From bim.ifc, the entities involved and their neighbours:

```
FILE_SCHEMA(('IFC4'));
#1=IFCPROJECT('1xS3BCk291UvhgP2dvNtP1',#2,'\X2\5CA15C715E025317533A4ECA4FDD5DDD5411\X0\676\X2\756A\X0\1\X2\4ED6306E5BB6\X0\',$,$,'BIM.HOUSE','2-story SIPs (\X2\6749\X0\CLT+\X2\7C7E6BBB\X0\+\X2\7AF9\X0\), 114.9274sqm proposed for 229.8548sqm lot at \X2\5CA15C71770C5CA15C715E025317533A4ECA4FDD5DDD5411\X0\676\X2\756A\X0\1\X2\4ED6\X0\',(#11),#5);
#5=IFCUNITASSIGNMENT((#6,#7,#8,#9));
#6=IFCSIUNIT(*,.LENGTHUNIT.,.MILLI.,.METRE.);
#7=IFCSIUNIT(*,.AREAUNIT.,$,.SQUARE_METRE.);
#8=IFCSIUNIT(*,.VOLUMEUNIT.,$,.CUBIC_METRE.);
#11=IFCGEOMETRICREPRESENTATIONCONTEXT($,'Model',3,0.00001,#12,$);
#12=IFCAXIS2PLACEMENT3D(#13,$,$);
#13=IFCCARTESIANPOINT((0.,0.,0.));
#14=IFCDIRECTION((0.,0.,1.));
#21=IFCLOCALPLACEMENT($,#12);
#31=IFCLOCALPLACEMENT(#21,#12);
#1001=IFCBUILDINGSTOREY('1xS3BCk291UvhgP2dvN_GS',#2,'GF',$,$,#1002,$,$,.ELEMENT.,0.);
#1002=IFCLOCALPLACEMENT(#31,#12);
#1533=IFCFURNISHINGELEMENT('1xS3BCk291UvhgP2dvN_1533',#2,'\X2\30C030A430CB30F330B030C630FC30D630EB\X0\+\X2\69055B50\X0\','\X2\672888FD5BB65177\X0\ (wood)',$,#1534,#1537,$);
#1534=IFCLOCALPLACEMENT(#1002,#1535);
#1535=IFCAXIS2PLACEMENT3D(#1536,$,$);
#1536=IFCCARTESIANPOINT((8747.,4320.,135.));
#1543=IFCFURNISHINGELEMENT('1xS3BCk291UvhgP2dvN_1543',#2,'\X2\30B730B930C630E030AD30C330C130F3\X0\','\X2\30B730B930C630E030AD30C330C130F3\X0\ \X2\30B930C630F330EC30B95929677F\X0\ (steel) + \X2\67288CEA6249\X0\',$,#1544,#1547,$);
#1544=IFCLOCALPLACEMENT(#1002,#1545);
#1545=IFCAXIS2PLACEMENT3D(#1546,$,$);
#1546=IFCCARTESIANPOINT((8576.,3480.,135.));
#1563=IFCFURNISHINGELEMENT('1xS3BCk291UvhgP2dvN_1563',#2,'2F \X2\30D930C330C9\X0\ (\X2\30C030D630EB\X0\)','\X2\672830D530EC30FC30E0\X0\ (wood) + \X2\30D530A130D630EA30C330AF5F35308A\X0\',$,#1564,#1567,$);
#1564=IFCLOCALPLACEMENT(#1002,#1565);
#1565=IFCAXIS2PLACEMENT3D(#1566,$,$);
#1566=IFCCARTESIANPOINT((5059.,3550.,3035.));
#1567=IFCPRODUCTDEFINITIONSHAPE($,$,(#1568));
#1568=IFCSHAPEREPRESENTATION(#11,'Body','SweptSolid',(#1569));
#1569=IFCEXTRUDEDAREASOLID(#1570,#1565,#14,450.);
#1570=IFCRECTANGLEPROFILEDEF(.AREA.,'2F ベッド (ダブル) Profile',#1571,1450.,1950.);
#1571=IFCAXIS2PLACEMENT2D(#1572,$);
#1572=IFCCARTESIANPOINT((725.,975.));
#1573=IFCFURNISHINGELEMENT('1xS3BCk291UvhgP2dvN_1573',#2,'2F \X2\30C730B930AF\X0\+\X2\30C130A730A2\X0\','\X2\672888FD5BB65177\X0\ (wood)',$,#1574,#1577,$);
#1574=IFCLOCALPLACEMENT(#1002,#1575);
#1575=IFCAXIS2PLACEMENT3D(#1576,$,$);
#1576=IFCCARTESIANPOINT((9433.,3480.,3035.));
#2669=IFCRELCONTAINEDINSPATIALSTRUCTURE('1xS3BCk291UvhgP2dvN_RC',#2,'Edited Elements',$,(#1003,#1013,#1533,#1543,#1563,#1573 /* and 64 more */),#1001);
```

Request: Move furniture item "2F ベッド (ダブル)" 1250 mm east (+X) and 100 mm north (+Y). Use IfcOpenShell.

```python
import ifcopenshell
import ifcopenshell.api.geometry
import ifcopenshell.util.placement
import ifcopenshell.util.unit

model = ifcopenshell.open("bim.ifc")
unit_scale = ifcopenshell.util.unit.calculate_unit_scale(model)

item = model.by_guid("1xS3BCk291UvhgP2dvN_1563")
matrix = ifcopenshell.util.placement.get_local_placement(item.ObjectPlacement)
matrix[0, 3] += 1.25 / unit_scale
matrix[1, 3] += 0.1 / unit_scale
ifcopenshell.api.geometry.edit_object_placement(model, product=item, matrix=matrix, is_si=False)

print(ifcopenshell.util.placement.get_local_placement(item.ObjectPlacement).round(3) + 0.0)

model.write("bim_edited.ifc")
```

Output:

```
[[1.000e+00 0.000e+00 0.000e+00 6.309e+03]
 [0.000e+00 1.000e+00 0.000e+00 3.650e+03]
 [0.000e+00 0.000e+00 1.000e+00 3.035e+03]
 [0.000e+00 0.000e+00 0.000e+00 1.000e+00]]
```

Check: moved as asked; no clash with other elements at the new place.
